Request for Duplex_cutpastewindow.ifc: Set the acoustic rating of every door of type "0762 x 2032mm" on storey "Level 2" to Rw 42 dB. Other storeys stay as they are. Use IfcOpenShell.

First a look at what the model holds.

```python
import ifcopenshell
import ifcopenshell.util.element

model = ifcopenshell.open("Duplex_cutpastewindow.ifc")
print(model.schema)
storey = next(s for s in model.by_type("IfcBuildingStorey") if s.Name == "Level 2")
doors = [e for e in ifcopenshell.util.element.get_decomposition(storey) if e.is_a("IfcDoor")]
seen = {}
for e in doors:
    element_type = ifcopenshell.util.element.get_type(e)
    key = (element_type.Name if element_type != e and element_type else None, ifcopenshell.util.element.get_pset(e, "Pset_DoorCommon", "AcousticRating"))
    seen[key] = seen.get(key, 0) + 1
for (name, value), count in sorted(seen.items(), key=str):
    print(count, "x", name, "|", value)
```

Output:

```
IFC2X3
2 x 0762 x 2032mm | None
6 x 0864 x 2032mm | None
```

```python
import ifcopenshell
import ifcopenshell.api.pset
import ifcopenshell.util.element

model = ifcopenshell.open("Duplex_cutpastewindow.ifc")

storey = next(s for s in model.by_type("IfcBuildingStorey") if s.Name == "Level 2")
doors = [e for e in ifcopenshell.util.element.get_decomposition(storey) if e.is_a("IfcDoor")]

count = 0
for e in doors:
    element_type = ifcopenshell.util.element.get_type(e)
    if element_type in (None, e) or element_type.Name != "0762 x 2032mm":
        continue
    # add_pset returns the element's existing set when there is one.
    pset = ifcopenshell.api.pset.add_pset(model, product=e, name="Pset_DoorCommon")
    ifcopenshell.api.pset.edit_pset(model, pset=pset, properties={"AcousticRating": "Rw 42 dB"})
    count += 1

print(count, "doors updated")

model.write("Duplex_cutpastewindow_v2.ifc")
```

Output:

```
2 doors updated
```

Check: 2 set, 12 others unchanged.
